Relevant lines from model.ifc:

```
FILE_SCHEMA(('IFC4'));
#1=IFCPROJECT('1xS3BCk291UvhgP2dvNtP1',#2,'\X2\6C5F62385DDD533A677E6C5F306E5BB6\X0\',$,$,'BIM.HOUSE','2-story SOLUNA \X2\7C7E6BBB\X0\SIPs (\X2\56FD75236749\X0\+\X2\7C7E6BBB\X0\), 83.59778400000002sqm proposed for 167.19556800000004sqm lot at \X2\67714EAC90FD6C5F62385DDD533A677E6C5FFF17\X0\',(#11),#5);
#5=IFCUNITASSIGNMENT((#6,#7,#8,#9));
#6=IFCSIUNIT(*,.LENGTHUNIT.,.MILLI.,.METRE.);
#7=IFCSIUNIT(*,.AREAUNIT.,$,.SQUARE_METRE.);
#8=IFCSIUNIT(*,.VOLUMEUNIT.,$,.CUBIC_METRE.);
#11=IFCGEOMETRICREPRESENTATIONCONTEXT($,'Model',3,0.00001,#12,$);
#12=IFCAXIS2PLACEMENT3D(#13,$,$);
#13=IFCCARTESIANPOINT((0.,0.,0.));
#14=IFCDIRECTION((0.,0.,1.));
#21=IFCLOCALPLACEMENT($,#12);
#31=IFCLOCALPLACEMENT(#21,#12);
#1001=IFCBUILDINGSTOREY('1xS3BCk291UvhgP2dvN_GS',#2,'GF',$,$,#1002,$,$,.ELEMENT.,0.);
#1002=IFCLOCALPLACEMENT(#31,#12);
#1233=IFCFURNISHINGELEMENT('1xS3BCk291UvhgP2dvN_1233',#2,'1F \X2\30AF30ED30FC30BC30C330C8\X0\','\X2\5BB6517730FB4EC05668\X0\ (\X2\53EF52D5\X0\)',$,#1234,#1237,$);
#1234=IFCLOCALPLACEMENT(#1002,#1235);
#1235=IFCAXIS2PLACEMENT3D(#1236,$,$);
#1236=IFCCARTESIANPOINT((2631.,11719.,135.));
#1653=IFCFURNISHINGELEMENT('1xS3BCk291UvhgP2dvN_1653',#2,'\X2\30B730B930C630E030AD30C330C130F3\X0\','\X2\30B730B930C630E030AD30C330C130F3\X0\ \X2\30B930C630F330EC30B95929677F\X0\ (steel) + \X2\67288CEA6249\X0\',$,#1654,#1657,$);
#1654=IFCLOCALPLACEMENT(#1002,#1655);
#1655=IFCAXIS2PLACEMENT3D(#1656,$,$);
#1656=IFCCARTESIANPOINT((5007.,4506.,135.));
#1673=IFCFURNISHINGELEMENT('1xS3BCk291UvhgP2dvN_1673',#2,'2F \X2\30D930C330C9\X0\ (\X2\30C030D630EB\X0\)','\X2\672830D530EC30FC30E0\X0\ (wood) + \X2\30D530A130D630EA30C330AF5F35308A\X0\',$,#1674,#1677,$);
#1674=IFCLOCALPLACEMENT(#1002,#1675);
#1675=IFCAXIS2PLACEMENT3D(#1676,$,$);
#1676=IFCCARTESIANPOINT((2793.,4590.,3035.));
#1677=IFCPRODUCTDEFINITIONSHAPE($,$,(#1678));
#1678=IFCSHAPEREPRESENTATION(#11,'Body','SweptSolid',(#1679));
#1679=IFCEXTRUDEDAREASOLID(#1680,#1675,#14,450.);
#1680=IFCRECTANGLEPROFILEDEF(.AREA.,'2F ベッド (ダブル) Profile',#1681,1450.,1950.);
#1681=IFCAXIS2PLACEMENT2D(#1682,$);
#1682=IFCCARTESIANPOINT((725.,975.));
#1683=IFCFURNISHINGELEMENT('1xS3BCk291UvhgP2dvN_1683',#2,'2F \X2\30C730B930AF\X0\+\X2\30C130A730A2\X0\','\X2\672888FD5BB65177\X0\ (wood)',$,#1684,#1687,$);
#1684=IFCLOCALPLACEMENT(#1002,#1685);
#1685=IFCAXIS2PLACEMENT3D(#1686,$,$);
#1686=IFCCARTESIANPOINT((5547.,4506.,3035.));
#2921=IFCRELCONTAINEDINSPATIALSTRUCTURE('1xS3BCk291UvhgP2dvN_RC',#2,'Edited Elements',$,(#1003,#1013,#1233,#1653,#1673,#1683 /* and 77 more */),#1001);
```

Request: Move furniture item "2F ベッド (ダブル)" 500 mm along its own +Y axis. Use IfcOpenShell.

```python
import ifcopenshell
import ifcopenshell.api.geometry
import ifcopenshell.util.placement
import ifcopenshell.util.unit

model = ifcopenshell.open("model.ifc")
unit_scale = ifcopenshell.util.unit.calculate_unit_scale(model)

item = model.by_id(1673)
matrix = ifcopenshell.util.placement.get_local_placement(item.ObjectPlacement)
matrix[:3, 3] += matrix[:3, 1] * 0.5 / unit_scale
ifcopenshell.api.geometry.edit_object_placement(model, product=item, matrix=matrix, is_si=False)

print(ifcopenshell.util.placement.get_local_placement(item.ObjectPlacement).round(3) + 0.0)

model.write("model_rev.ifc")
```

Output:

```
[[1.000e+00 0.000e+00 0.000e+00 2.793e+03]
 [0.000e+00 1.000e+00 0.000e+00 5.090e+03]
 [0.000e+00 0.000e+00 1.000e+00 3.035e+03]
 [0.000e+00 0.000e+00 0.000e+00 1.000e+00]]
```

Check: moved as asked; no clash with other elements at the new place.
